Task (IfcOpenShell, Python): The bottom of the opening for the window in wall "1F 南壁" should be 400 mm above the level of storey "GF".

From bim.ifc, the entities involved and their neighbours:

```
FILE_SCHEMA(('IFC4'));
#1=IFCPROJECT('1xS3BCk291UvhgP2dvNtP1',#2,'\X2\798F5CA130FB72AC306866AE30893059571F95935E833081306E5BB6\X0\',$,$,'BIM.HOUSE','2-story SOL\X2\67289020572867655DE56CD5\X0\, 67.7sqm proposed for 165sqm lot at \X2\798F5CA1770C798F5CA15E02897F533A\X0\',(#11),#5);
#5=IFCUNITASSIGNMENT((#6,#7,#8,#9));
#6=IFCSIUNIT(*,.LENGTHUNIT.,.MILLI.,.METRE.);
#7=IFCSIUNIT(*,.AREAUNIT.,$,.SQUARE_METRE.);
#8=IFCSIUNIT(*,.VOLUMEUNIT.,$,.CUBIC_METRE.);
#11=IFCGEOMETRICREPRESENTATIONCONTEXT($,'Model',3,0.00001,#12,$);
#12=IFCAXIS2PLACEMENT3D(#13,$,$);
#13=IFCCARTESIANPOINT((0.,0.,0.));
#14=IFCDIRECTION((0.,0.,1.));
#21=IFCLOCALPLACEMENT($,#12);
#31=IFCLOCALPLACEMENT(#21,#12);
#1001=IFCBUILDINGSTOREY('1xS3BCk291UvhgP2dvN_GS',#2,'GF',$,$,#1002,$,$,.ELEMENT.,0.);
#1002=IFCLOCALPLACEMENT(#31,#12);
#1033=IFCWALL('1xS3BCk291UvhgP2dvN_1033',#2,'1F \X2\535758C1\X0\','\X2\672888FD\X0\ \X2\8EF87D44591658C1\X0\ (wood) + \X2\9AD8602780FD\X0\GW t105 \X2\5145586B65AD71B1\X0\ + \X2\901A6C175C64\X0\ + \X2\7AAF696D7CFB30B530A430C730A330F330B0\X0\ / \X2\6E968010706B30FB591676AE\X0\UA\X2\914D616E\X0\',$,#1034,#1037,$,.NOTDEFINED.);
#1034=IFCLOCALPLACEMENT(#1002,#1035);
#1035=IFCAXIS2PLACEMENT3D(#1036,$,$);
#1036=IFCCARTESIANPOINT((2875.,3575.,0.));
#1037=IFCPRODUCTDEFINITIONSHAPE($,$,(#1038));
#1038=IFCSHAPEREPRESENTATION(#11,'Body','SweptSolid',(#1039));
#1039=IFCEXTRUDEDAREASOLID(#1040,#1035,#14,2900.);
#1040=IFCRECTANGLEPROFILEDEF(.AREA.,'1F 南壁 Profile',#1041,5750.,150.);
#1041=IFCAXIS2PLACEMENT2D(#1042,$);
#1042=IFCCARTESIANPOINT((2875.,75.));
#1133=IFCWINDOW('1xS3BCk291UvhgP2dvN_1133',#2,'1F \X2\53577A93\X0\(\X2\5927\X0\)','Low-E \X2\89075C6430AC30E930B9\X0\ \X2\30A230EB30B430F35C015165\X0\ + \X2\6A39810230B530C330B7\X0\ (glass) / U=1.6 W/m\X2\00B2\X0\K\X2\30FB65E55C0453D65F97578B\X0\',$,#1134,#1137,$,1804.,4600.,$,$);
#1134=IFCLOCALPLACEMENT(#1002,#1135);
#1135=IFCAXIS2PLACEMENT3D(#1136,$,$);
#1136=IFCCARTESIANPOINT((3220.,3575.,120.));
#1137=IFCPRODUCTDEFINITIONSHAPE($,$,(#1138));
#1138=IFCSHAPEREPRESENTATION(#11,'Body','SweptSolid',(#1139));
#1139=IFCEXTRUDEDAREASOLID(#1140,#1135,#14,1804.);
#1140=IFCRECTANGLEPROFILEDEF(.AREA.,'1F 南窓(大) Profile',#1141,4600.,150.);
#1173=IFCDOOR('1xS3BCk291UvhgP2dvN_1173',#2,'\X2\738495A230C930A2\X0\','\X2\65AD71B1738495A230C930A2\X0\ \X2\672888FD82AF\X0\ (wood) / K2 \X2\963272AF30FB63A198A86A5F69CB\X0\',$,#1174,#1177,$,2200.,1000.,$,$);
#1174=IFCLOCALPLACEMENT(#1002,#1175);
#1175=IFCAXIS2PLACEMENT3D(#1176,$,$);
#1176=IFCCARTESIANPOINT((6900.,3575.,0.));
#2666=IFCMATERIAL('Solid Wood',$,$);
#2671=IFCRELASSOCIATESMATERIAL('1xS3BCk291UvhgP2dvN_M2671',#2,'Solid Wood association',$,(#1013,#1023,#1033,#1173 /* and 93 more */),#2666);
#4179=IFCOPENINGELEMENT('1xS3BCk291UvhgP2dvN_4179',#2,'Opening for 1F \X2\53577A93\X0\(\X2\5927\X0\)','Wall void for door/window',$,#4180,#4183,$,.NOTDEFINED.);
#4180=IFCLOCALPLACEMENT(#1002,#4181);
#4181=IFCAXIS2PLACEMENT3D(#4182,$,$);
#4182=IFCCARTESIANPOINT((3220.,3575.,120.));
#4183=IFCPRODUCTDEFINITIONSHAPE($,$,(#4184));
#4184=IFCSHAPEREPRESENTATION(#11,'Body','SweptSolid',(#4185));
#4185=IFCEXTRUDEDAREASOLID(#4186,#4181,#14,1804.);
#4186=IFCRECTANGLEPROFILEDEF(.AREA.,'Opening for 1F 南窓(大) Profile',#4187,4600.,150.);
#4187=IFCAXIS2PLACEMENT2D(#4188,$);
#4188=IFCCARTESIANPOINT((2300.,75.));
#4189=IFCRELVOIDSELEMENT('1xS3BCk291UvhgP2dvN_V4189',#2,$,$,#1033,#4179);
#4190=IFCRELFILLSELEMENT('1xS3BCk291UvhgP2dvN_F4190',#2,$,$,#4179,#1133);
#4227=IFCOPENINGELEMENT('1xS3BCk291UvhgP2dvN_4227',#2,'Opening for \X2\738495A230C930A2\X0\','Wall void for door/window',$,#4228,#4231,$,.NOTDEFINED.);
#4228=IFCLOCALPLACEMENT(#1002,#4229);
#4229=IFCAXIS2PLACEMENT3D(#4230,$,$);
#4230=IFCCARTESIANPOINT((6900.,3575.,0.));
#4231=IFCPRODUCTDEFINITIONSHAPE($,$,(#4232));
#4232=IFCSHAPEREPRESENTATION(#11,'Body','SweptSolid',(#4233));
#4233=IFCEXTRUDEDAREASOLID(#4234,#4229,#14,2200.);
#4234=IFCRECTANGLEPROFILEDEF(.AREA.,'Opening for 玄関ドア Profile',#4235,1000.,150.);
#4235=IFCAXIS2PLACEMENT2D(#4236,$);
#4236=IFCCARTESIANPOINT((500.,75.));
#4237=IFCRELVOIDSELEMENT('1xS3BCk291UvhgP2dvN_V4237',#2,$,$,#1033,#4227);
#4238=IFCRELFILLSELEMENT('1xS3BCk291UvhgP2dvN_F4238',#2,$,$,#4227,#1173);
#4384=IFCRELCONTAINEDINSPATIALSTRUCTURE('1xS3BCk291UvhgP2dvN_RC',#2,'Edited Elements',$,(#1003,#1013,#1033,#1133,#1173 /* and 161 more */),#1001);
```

```python
import numpy as np
import ifcopenshell
import ifcopenshell.api.geometry
import ifcopenshell.geom
import ifcopenshell.util.element
import ifcopenshell.util.placement
import ifcopenshell.util.shape
import ifcopenshell.util.unit

model = ifcopenshell.open("bim.ifc")
unit_scale = ifcopenshell.util.unit.calculate_unit_scale(model)

window = model.by_id(1133)
opening = window.FillsVoids[0].RelatingOpeningElement
storey = ifcopenshell.util.element.get_container(window, ifc_class="IfcBuildingStorey")
level = ifcopenshell.util.placement.get_local_placement(storey.ObjectPlacement)[2, 3]

# The opening's origin need not be at the sill, so measure its lowest point.
shape = ifcopenshell.geom.create_shape(ifcopenshell.geom.settings(), opening)
bottom = ifcopenshell.util.shape.get_shape_bottom_elevation(shape, shape.geometry) / unit_scale
dz = level + 400.0 - bottom

shift = np.array([0.0, 0.0, dz])
# The window is not placed relative to its opening, so move both.
for product in (opening, window):
    matrix = ifcopenshell.util.placement.get_local_placement(product.ObjectPlacement)
    matrix[:3, 3] += shift
    ifcopenshell.api.geometry.edit_object_placement(model, product=product, matrix=matrix, is_si=False)

print(f"moved by {dz * unit_scale:+.3f} m")

model.write("bim_edited.ifc")
```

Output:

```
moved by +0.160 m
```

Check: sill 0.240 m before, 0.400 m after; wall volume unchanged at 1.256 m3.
